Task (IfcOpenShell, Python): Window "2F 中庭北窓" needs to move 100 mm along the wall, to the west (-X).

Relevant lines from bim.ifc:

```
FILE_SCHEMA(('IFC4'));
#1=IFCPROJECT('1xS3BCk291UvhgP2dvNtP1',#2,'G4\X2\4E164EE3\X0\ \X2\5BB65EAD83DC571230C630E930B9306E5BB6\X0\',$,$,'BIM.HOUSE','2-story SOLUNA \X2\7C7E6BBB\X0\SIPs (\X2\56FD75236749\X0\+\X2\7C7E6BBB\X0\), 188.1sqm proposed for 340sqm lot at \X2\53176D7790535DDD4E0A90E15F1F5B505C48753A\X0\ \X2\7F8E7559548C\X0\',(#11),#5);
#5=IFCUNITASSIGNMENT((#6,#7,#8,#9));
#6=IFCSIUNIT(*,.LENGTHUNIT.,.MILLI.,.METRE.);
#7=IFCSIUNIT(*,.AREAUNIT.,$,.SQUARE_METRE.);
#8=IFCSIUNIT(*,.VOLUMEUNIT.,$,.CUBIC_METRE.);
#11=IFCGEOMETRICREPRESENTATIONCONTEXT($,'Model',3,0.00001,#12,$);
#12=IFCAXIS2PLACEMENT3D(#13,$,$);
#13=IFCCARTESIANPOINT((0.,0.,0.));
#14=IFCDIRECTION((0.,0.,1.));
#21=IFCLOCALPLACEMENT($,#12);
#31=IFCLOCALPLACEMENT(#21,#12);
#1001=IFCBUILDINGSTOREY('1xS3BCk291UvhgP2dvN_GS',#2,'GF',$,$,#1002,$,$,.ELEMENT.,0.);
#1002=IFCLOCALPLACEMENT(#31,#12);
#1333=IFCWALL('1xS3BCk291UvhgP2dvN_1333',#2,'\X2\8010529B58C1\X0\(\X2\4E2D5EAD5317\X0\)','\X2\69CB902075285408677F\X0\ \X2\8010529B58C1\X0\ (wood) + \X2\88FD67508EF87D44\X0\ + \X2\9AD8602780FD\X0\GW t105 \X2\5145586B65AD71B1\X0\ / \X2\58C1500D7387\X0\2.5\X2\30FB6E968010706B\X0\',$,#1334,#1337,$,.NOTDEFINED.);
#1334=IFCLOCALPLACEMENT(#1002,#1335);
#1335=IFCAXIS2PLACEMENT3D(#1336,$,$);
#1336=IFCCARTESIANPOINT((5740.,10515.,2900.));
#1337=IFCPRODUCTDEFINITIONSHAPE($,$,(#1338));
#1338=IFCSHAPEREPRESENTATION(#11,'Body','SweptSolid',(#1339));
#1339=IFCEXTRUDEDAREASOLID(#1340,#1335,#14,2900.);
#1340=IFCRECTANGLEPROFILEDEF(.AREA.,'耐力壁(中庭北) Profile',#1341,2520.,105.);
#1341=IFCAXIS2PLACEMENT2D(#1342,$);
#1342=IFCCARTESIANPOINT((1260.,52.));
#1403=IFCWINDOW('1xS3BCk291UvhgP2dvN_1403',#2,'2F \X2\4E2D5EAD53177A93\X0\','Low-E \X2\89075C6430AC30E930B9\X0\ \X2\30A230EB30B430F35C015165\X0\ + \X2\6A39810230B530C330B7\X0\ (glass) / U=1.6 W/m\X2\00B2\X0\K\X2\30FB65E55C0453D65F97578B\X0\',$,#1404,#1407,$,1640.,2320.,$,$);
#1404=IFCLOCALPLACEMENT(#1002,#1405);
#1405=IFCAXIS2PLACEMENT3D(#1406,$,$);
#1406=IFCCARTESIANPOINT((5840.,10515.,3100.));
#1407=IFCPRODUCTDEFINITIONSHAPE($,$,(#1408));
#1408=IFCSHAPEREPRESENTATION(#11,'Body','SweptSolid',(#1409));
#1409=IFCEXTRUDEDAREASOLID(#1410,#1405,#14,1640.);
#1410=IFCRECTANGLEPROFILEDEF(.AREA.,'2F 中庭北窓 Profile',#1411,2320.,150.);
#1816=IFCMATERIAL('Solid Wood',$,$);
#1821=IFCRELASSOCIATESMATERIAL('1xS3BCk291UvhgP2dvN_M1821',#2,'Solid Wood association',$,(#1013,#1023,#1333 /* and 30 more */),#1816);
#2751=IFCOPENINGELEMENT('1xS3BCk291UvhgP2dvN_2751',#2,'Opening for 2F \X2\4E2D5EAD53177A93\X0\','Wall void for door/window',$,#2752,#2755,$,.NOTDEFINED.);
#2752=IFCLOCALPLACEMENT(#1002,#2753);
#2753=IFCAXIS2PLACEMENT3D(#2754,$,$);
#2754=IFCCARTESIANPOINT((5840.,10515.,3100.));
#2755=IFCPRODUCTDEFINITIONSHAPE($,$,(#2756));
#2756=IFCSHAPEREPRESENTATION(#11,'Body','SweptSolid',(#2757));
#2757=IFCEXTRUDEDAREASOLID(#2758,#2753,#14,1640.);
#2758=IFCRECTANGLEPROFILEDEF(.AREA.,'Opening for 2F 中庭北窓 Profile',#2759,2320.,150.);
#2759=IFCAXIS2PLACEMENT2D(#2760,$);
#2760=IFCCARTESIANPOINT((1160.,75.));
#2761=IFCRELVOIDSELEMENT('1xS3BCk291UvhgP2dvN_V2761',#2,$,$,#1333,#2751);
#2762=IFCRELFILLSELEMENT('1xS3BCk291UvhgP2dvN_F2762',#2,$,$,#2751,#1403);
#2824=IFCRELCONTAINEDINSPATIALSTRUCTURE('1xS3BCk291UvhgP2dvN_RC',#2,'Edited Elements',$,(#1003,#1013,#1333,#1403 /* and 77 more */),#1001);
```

```python
import ifcopenshell
import ifcopenshell.api.geometry
import ifcopenshell.util.placement
import ifcopenshell.util.unit

model = ifcopenshell.open("bim.ifc")
unit_scale = ifcopenshell.util.unit.calculate_unit_scale(model)

window = model.by_guid("1xS3BCk291UvhgP2dvN_1403")
opening = window.FillsVoids[0].RelatingOpeningElement
wall = opening.VoidsElements[0].RelatingBuildingElement

wall_matrix = ifcopenshell.util.placement.get_local_placement(wall.ObjectPlacement)
shift = wall_matrix[:3, 0] * -0.1 / unit_scale
before = ifcopenshell.util.placement.get_local_placement(window.ObjectPlacement)[:3, 3].copy()

# The window is not placed relative to its opening, so move both.
for product in (opening, window):
    matrix = ifcopenshell.util.placement.get_local_placement(product.ObjectPlacement)
    matrix[:3, 3] += shift
    ifcopenshell.api.geometry.edit_object_placement(model, product=product, matrix=matrix, is_si=False)

after = ifcopenshell.util.placement.get_local_placement(window.ObjectPlacement)[:3, 3]
print("window moved by", (after - before).round(3) + 0.0)

model.write("bim_v2.ifc")
```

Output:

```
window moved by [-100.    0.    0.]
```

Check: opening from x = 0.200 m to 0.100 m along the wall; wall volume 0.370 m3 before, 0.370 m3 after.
